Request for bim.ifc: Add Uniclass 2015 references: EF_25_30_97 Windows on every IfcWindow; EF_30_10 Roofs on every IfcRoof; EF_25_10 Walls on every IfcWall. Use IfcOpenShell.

First a look at what the model holds.

```python
import ifcopenshell

model = ifcopenshell.open("bim.ifc")
print(model.schema)
print("classifications:", [c.Name for c in model.by_type("IfcClassification")])
for ifc_class in ("IfcDoor", "IfcRoof", "IfcStair", "IfcWall", "IfcWindow"):
    print(ifc_class, len(model.by_type(ifc_class)))
```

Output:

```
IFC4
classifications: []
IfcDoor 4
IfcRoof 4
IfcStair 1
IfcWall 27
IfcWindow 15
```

```python
import ifcopenshell
import ifcopenshell.api.classification

model = ifcopenshell.open("bim.ifc")

system = ifcopenshell.api.classification.add_classification(model, classification="Uniclass 2015")

codes = {
    "IfcWindow": ("EF_25_30_97", "Windows"),
    "IfcRoof": ("EF_30_10", "Roofs"),
    "IfcWall": ("EF_25_10", "Walls"),
}
for ifc_class, (code, name) in codes.items():
    products = model.by_type(ifc_class)
    ifcopenshell.api.classification.add_reference(
        model, products=products, classification=system, identification=code, name=name
    )
    print(code, len(products))

model.write("bim_v2.ifc")
```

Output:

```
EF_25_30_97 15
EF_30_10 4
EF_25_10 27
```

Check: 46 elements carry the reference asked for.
